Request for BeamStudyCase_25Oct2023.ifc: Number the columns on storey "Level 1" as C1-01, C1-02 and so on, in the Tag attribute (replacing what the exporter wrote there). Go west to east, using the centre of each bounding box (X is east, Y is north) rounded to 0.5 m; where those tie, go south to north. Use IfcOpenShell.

First a look at what the model holds.

```python
import ifcopenshell
import ifcopenshell.util.element
import ifcopenshell.util.placement

model = ifcopenshell.open("BeamStudyCase_25Oct2023.ifc")
print(model.schema)
storey = next(s for s in model.by_type("IfcBuildingStorey") if s.Name == "Level 1")
columns = [e for e in ifcopenshell.util.element.get_decomposition(storey) if e.is_a("IfcColumn")]
for e in sorted(columns, key=lambda e: e.id()):
    origin = ifcopenshell.util.placement.get_local_placement(e.ObjectPlacement)[:3, 3]
    print(e.id(), e.Tag, e.Name, origin.round(2) + 0.0, sep=" | ")
```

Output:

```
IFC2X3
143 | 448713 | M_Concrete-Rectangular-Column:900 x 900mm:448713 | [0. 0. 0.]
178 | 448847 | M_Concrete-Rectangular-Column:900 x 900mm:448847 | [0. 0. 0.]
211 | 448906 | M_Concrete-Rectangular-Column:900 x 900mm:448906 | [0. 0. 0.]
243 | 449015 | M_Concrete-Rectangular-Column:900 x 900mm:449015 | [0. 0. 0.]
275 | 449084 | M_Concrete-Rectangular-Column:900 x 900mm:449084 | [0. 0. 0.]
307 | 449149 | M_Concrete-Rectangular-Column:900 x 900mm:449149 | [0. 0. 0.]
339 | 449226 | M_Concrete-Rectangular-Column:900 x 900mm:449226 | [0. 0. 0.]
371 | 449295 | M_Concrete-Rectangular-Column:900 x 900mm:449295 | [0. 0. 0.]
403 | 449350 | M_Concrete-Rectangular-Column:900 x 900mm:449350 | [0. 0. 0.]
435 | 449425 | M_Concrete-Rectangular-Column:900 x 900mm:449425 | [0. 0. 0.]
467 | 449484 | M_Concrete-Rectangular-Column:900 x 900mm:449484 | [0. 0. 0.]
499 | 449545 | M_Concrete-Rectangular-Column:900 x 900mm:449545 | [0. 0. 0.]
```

```python
import ifcopenshell
import ifcopenshell.geom
import ifcopenshell.util.element
import ifcopenshell.util.shape

model = ifcopenshell.open("BeamStudyCase_25Oct2023.ifc")
settings = ifcopenshell.geom.settings()
settings.set("use-world-coords", True)


def centre(element):
    shape = ifcopenshell.geom.create_shape(settings, element)
    return ifcopenshell.util.shape.get_bbox_centroid(shape.geometry)


storey = next(s for s in model.by_type("IfcBuildingStorey") if s.Name == "Level 1")
columns = [e for e in ifcopenshell.util.element.get_decomposition(storey) if e.is_a("IfcColumn")]

# Insertion points can sit at a corner or the storey origin, so sort by the geometry (in metres).
centres = {e: centre(e) for e in columns}
columns.sort(key=lambda e: (round(centres[e][0] / 0.5), centres[e][1]))

for i, e in enumerate(columns, start=1):
    number = f"C1-{i:02d}"
    e.Tag = number
    print(e.id(), number)

model.write("BeamStudyCase_25Oct2023_edited.ifc")
```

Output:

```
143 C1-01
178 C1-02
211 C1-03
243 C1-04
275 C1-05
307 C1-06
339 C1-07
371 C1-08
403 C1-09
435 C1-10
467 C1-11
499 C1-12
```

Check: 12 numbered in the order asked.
